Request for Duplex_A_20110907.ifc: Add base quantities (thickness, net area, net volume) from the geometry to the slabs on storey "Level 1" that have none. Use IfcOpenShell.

First a look at what the model holds.

```python
import ifcopenshell
import ifcopenshell.util.element
import ifcopenshell.util.unit

model = ifcopenshell.open("Duplex_A_20110907.ifc")
print(model.schema)
for unit_type in ("LENGTHUNIT", "AREAUNIT", "VOLUMEUNIT"):
    print(unit_type, ifcopenshell.util.unit.calculate_unit_scale(model, unit_type))
storey = next(s for s in model.by_type("IfcBuildingStorey") if s.Name == "Level 1")
slabs = [e for e in ifcopenshell.util.element.get_decomposition(storey) if e.is_a("IfcSlab")]
for e in sorted(slabs, key=lambda e: e.id()):
    print(e.id(), e.is_a(), e.Name, list(ifcopenshell.util.element.get_psets(e, qtos_only=True)), sep=" | ")
```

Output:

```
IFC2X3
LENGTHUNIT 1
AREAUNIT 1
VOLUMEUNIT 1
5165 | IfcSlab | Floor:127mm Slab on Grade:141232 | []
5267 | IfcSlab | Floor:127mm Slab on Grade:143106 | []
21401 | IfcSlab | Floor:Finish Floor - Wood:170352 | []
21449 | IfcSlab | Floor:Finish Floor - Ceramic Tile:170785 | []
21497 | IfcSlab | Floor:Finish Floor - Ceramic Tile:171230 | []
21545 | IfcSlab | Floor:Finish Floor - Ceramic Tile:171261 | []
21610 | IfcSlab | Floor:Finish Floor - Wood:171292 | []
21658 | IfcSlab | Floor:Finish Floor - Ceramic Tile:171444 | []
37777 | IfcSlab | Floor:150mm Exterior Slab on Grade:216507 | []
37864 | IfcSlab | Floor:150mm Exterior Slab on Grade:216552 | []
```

```python
import ifcopenshell
import ifcopenshell.api.pset
import ifcopenshell.geom
import ifcopenshell.util.element
import ifcopenshell.util.shape
import ifcopenshell.util.unit

model = ifcopenshell.open("Duplex_A_20110907.ifc")
unit_scale = ifcopenshell.util.unit.calculate_unit_scale(model)
area_scale = ifcopenshell.util.unit.calculate_unit_scale(model, "AREAUNIT")
volume_scale = ifcopenshell.util.unit.calculate_unit_scale(model, "VOLUMEUNIT")
settings = ifcopenshell.geom.settings()

storey = next(s for s in model.by_type("IfcBuildingStorey") if s.Name == "Level 1")
slabs = [e for e in ifcopenshell.util.element.get_decomposition(storey) if e.is_a("IfcSlab")]

for e in sorted(slabs, key=lambda e: e.id()):
    if ifcopenshell.util.element.get_psets(e, qtos_only=True, should_inherit=False):
        continue
    # Geometry comes back in metres, in the element's own axes.
    shape = ifcopenshell.geom.create_shape(settings, e)
    values = {
        "Width": ifcopenshell.util.shape.get_z(shape.geometry) / unit_scale,
        "NetArea": ifcopenshell.util.shape.get_footprint_area(shape.geometry) / area_scale,
        "NetVolume": ifcopenshell.util.shape.get_volume(shape.geometry) / volume_scale,
    }
    qto = ifcopenshell.api.pset.add_qto(model, product=e, name="BaseQuantities")
    ifcopenshell.api.pset.edit_qto(model, qto=qto, properties=values)
    print(e.id(), {k: round(v, 3) for k, v in values.items()})

model.write("Duplex_A_20110907_updated.ifc")
```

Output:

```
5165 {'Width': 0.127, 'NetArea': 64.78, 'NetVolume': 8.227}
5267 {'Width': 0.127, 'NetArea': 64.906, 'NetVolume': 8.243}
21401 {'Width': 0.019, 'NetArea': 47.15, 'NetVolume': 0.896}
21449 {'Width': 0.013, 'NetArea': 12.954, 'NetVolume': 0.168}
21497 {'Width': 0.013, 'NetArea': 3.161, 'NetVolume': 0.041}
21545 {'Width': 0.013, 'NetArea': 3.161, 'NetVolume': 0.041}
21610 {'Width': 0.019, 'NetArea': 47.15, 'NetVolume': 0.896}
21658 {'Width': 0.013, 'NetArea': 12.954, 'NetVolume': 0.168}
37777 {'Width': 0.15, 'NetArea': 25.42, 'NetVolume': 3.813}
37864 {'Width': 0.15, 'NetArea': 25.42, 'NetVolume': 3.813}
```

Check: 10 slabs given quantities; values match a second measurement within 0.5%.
